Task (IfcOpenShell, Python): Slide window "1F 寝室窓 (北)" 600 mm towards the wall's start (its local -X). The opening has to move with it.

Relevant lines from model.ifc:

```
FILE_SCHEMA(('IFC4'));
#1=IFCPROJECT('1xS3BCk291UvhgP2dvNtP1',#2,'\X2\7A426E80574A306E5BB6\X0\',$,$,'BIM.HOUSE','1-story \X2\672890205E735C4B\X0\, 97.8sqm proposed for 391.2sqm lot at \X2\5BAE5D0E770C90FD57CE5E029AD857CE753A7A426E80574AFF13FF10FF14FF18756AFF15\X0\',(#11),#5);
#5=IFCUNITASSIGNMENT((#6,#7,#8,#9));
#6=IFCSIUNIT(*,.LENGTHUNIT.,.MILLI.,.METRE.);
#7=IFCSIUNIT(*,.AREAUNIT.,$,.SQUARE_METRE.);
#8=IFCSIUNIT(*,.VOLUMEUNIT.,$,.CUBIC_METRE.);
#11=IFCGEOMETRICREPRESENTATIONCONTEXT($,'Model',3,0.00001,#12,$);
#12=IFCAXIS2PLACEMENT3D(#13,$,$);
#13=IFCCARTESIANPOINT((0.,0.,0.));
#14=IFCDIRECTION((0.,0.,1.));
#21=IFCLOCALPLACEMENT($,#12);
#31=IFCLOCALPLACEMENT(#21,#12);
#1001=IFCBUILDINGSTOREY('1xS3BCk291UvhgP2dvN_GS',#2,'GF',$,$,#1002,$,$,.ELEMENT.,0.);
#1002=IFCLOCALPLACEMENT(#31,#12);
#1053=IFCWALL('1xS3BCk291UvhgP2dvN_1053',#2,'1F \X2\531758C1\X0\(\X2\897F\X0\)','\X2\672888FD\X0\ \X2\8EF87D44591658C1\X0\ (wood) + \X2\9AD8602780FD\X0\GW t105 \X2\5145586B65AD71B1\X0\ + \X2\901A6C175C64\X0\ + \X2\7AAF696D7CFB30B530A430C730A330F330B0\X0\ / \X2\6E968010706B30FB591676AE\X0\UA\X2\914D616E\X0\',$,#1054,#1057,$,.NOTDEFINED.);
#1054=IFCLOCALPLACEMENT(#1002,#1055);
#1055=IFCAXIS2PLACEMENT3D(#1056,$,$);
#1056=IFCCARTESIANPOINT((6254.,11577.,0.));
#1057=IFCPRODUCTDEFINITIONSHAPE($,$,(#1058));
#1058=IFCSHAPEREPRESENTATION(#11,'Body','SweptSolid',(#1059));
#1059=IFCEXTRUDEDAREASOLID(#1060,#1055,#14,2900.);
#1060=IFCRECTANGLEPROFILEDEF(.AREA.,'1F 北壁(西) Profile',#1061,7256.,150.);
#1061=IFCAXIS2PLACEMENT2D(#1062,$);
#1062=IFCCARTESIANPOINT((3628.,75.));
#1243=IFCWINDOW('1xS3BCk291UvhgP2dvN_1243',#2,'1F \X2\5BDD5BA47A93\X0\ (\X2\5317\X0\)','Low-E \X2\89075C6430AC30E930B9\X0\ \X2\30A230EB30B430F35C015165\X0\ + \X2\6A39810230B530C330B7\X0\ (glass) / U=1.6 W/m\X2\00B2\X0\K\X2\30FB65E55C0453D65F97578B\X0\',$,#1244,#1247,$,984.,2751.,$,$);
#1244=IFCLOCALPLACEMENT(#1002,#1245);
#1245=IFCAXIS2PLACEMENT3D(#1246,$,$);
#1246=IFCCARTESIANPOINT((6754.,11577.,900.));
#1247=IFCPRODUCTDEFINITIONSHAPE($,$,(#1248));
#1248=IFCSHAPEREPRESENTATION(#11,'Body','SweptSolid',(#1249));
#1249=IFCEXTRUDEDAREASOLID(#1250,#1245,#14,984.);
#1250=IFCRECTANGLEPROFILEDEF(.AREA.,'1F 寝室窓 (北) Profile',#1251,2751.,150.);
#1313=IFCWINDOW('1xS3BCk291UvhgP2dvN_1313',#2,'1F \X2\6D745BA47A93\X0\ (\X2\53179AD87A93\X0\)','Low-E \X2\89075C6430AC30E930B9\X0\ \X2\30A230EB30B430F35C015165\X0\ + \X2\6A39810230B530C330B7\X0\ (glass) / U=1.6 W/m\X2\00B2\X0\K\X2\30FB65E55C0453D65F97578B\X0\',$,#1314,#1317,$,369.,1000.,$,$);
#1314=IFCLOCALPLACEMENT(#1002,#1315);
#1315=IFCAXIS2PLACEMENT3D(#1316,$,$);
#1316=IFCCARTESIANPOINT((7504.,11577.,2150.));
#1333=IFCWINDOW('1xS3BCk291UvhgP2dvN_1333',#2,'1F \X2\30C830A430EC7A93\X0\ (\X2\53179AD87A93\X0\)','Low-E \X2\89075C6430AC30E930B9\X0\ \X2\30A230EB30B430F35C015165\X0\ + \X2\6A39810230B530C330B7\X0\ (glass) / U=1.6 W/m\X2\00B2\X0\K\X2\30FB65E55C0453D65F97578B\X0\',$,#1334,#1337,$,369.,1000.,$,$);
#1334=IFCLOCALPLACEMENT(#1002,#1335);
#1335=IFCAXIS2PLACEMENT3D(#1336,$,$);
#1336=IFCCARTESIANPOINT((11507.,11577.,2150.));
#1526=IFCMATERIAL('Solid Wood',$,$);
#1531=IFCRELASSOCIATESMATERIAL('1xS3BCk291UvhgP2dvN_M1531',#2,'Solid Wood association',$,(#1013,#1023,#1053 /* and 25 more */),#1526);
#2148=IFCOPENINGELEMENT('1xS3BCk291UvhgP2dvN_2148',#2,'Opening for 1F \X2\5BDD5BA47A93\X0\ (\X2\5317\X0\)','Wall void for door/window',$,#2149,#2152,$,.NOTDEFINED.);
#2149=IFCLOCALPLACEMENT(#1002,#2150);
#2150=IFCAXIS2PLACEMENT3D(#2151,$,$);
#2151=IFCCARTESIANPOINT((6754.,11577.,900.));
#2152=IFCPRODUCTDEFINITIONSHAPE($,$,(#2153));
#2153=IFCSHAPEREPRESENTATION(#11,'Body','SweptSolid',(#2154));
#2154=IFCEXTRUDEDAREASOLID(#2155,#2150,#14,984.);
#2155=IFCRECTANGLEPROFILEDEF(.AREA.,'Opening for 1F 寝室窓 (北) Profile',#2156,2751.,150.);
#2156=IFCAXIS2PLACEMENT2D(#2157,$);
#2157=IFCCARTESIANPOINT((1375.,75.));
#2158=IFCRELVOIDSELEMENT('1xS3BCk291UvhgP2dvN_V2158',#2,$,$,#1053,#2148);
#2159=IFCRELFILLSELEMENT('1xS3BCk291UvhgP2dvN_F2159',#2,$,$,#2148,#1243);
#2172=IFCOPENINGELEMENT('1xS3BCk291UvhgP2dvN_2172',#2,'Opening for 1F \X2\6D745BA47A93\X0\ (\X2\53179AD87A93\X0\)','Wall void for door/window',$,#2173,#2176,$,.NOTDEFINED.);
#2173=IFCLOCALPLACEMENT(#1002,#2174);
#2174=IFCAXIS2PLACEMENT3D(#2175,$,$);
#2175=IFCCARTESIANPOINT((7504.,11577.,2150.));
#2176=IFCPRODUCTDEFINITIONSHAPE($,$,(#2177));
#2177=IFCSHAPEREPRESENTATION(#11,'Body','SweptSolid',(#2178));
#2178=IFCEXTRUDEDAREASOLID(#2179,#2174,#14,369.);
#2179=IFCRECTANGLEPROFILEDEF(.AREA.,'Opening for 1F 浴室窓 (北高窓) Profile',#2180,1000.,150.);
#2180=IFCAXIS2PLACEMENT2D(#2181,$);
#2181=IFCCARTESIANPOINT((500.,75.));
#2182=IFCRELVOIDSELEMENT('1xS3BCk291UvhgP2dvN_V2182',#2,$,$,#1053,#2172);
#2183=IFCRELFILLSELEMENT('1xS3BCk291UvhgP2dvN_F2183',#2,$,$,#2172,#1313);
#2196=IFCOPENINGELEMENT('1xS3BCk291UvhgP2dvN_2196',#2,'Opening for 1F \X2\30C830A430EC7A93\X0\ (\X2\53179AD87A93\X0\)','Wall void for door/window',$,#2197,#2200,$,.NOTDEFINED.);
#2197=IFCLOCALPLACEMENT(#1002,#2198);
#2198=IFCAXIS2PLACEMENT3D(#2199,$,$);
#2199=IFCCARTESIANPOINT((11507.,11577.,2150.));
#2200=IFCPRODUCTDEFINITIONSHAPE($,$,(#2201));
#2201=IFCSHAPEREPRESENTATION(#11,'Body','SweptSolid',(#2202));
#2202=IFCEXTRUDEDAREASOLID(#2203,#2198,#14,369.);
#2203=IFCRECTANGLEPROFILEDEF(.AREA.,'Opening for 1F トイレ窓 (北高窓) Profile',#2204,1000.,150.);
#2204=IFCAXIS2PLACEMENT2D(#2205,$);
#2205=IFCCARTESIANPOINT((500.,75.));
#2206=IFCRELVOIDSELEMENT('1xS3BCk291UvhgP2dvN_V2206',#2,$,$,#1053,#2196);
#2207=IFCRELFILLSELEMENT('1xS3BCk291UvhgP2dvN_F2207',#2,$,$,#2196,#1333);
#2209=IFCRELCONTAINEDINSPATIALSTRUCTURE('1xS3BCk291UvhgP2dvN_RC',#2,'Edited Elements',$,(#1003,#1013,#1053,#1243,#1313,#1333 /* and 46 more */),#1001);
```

```python
import ifcopenshell
import ifcopenshell.api.geometry
import ifcopenshell.util.placement
import ifcopenshell.util.unit

model = ifcopenshell.open("model.ifc")
unit_scale = ifcopenshell.util.unit.calculate_unit_scale(model)

window = model.by_id(1243)
opening = window.FillsVoids[0].RelatingOpeningElement
wall = opening.VoidsElements[0].RelatingBuildingElement

wall_matrix = ifcopenshell.util.placement.get_local_placement(wall.ObjectPlacement)
shift = wall_matrix[:3, 0] * -0.6 / unit_scale
before = ifcopenshell.util.placement.get_local_placement(window.ObjectPlacement)[:3, 3].copy()

# The window is not placed relative to its opening, so move both.
for product in (opening, window):
    matrix = ifcopenshell.util.placement.get_local_placement(product.ObjectPlacement)
    matrix[:3, 3] += shift
    ifcopenshell.api.geometry.edit_object_placement(model, product=product, matrix=matrix, is_si=False)

after = ifcopenshell.util.placement.get_local_placement(window.ObjectPlacement)[:3, 3]
print("window moved by", (after - before).round(3) + 0.0)

model.write("model_updated.ifc")
```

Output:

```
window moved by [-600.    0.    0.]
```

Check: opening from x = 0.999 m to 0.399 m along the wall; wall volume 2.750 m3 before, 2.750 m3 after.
